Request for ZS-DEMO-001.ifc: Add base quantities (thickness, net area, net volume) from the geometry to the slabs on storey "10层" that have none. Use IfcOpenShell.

First a look at what the model holds.

```python
import ifcopenshell
import ifcopenshell.util.element
import ifcopenshell.util.unit

model = ifcopenshell.open("ZS-DEMO-001.ifc")
print(model.schema)
for unit_type in ("LENGTHUNIT", "AREAUNIT", "VOLUMEUNIT"):
    print(unit_type, ifcopenshell.util.unit.calculate_unit_scale(model, unit_type))
storey = next(s for s in model.by_type("IfcBuildingStorey") if s.Name == "10层")
slabs = [e for e in ifcopenshell.util.element.get_decomposition(storey) if e.is_a("IfcSlab")]
for e in sorted(slabs, key=lambda e: e.id()):
    print(e.id(), e.is_a(), e.Name, list(ifcopenshell.util.element.get_psets(e, qtos_only=True)), sep=" | ")
```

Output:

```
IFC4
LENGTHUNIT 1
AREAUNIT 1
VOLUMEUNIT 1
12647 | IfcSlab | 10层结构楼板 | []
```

```python
import ifcopenshell
import ifcopenshell.api.pset
import ifcopenshell.geom
import ifcopenshell.util.element
import ifcopenshell.util.shape
import ifcopenshell.util.unit

model = ifcopenshell.open("ZS-DEMO-001.ifc")
unit_scale = ifcopenshell.util.unit.calculate_unit_scale(model)
area_scale = ifcopenshell.util.unit.calculate_unit_scale(model, "AREAUNIT")
volume_scale = ifcopenshell.util.unit.calculate_unit_scale(model, "VOLUMEUNIT")
settings = ifcopenshell.geom.settings()

storey = next(s for s in model.by_type("IfcBuildingStorey") if s.Name == "10层")
slabs = [e for e in ifcopenshell.util.element.get_decomposition(storey) if e.is_a("IfcSlab")]

for e in sorted(slabs, key=lambda e: e.id()):
    if ifcopenshell.util.element.get_psets(e, qtos_only=True, should_inherit=False):
        continue
    # Geometry comes back in metres, in the element's own axes.
    shape = ifcopenshell.geom.create_shape(settings, e)
    values = {
        "Width": ifcopenshell.util.shape.get_z(shape.geometry) / unit_scale,
        "NetArea": ifcopenshell.util.shape.get_footprint_area(shape.geometry) / area_scale,
        "NetVolume": ifcopenshell.util.shape.get_volume(shape.geometry) / volume_scale,
    }
    qto = ifcopenshell.api.pset.add_qto(model, product=e, name="Qto_SlabBaseQuantities")
    ifcopenshell.api.pset.edit_qto(model, qto=qto, properties=values)
    print(e.id(), {k: round(v, 3) for k, v in values.items()})

model.write("ZS-DEMO-001_updated.ifc")
```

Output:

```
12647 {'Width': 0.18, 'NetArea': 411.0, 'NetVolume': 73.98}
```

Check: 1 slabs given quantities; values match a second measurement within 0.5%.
